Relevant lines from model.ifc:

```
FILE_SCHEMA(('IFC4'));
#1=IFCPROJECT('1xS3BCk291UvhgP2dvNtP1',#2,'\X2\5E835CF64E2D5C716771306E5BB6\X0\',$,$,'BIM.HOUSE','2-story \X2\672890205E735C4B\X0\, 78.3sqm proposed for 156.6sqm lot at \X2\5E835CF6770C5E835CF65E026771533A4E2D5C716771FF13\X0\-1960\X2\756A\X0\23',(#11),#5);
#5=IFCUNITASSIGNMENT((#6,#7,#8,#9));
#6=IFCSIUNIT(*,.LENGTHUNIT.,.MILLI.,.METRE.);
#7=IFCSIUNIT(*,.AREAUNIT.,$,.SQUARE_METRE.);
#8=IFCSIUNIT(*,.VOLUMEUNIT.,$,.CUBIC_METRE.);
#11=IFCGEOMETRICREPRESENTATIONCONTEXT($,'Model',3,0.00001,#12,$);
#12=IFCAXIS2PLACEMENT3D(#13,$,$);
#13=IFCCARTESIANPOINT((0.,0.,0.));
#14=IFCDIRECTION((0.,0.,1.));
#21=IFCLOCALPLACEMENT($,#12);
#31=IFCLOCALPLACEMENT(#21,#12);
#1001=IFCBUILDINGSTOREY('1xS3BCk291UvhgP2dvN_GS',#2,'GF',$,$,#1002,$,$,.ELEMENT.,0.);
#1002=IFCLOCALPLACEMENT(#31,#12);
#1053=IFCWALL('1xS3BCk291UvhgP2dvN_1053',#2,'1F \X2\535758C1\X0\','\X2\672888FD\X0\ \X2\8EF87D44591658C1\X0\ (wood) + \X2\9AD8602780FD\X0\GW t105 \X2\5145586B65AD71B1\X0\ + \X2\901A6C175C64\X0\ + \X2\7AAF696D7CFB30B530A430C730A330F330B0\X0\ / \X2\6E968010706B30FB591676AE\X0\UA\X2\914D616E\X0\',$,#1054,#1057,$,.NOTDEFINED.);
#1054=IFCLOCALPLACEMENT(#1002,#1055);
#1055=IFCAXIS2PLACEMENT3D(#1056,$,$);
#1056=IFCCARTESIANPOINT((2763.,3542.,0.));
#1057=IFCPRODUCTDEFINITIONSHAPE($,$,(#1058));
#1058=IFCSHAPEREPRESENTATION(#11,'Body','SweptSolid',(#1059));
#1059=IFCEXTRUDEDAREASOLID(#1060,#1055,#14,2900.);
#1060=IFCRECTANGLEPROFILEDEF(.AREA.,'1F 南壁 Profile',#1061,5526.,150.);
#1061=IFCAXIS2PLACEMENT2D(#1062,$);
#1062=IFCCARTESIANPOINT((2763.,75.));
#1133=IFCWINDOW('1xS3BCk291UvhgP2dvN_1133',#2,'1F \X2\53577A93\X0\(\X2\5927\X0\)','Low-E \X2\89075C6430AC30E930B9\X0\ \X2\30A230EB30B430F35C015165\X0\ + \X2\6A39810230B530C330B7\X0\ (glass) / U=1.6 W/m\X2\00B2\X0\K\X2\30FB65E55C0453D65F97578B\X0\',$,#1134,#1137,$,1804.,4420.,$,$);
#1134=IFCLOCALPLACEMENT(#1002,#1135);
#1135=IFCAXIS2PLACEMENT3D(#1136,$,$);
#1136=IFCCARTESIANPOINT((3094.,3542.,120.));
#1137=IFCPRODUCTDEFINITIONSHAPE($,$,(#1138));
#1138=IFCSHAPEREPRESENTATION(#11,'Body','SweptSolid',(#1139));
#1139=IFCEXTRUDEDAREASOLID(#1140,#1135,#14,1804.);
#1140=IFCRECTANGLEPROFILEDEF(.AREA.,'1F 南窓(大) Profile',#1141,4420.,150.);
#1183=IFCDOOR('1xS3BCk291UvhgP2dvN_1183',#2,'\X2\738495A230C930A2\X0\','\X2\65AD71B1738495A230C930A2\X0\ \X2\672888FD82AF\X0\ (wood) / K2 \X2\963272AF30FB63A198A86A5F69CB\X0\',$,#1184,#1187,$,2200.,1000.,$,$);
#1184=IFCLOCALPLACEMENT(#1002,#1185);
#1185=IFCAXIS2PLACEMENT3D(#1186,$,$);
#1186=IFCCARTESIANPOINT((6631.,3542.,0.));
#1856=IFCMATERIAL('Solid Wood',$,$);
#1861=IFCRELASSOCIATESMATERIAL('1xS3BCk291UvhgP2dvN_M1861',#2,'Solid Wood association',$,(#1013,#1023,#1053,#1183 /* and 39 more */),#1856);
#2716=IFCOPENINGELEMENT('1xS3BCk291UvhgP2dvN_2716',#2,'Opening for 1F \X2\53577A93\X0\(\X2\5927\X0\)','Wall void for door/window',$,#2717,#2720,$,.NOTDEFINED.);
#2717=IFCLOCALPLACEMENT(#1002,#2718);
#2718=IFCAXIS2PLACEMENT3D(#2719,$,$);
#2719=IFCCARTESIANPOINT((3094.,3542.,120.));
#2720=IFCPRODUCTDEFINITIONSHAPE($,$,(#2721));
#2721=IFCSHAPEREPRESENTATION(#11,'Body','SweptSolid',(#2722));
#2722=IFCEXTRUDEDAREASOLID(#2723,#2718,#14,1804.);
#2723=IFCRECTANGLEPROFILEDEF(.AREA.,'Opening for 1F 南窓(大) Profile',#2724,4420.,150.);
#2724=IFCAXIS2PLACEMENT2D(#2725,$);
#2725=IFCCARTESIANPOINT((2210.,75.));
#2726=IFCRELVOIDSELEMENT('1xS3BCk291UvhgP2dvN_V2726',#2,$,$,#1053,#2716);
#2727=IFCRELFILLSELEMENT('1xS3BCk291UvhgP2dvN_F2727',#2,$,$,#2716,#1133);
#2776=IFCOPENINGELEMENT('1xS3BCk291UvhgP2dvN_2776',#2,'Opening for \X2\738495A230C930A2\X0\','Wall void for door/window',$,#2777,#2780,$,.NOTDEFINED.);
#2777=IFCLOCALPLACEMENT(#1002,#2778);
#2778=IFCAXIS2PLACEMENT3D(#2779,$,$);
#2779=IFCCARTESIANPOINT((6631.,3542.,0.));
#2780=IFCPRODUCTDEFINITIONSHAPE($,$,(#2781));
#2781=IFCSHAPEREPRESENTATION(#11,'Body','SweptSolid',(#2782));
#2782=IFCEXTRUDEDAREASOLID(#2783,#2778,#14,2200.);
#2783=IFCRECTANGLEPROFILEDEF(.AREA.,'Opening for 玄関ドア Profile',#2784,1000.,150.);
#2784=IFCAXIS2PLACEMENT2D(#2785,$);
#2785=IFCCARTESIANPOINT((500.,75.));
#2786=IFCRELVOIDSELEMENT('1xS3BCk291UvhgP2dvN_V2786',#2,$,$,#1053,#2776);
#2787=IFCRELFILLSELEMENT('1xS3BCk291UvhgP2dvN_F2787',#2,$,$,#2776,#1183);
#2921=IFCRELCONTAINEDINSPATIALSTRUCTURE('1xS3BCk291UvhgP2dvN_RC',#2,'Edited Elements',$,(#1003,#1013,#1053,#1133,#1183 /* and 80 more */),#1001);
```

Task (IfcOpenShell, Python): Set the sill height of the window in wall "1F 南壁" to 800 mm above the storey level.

```python
import numpy as np
import ifcopenshell
import ifcopenshell.api.geometry
import ifcopenshell.geom
import ifcopenshell.util.element
import ifcopenshell.util.placement
import ifcopenshell.util.shape
import ifcopenshell.util.unit

model = ifcopenshell.open("model.ifc")
unit_scale = ifcopenshell.util.unit.calculate_unit_scale(model)

window = model.by_guid("1xS3BCk291UvhgP2dvN_1133")
opening = window.FillsVoids[0].RelatingOpeningElement
storey = ifcopenshell.util.element.get_container(window, ifc_class="IfcBuildingStorey")
level = ifcopenshell.util.placement.get_local_placement(storey.ObjectPlacement)[2, 3]

# The opening's origin need not be at the sill, so measure its lowest point.
shape = ifcopenshell.geom.create_shape(ifcopenshell.geom.settings(), opening)
bottom = ifcopenshell.util.shape.get_shape_bottom_elevation(shape, shape.geometry) / unit_scale
dz = level + 0.8 / unit_scale - bottom

shift = np.array([0.0, 0.0, dz])
# The window is not placed relative to its opening, so move both.
for product in (opening, window):
    matrix = ifcopenshell.util.placement.get_local_placement(product.ObjectPlacement)
    matrix[:3, 3] += shift
    ifcopenshell.api.geometry.edit_object_placement(model, product=product, matrix=matrix, is_si=False)

print(f"moved by {dz * unit_scale:+.3f} m")

model.write("model_rev.ifc")
```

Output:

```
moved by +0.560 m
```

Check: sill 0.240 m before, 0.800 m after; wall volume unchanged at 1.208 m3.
